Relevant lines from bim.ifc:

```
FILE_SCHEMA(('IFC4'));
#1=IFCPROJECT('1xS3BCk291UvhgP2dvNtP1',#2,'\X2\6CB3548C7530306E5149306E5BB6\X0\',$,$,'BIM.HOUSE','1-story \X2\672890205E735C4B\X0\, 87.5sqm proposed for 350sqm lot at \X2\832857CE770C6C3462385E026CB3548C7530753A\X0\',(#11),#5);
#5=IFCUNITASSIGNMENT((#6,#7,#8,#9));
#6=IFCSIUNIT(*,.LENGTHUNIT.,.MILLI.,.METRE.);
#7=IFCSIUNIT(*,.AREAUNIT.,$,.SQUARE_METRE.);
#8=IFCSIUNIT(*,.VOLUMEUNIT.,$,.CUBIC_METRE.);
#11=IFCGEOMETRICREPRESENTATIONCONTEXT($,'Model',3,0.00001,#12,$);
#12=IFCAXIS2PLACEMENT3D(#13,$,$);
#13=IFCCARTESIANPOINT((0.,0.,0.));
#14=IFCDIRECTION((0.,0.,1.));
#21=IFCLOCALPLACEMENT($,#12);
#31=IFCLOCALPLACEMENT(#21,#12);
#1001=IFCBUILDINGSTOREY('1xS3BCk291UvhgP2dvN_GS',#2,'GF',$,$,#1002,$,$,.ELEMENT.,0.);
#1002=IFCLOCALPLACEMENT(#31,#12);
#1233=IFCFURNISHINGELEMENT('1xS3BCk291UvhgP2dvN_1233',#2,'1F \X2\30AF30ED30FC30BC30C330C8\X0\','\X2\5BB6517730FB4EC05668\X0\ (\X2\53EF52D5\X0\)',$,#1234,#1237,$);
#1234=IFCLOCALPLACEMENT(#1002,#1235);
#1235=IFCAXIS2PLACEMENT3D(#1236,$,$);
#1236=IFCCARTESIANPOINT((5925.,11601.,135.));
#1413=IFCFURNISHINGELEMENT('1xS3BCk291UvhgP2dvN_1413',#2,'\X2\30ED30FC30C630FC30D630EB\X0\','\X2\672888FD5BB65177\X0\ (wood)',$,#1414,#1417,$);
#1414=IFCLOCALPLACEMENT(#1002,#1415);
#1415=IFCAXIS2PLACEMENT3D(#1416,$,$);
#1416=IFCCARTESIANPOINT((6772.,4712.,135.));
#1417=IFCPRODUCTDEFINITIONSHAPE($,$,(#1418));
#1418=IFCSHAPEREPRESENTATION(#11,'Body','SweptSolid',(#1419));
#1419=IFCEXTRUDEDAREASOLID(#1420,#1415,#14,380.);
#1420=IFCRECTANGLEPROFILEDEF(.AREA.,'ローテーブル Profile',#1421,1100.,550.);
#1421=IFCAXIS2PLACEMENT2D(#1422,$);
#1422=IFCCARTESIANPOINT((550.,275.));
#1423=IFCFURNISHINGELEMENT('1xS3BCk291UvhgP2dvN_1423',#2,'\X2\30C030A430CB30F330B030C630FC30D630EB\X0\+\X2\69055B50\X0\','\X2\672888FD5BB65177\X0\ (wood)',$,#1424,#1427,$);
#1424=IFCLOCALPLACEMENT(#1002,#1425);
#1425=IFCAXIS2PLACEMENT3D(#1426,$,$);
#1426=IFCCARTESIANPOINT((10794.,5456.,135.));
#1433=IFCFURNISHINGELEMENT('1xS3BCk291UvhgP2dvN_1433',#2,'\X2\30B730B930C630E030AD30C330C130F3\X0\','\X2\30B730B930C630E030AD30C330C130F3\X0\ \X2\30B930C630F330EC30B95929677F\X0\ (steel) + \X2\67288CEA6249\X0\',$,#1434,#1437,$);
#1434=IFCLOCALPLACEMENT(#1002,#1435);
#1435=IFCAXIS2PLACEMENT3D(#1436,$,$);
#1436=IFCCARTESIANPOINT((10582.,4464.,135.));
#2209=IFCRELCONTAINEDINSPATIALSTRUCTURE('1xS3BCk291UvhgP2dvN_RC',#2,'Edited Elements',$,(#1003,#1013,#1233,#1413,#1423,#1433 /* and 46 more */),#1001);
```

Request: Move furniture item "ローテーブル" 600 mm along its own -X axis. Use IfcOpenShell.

```python
import ifcopenshell
import ifcopenshell.api.geometry
import ifcopenshell.util.placement
import ifcopenshell.util.unit

model = ifcopenshell.open("bim.ifc")
unit_scale = ifcopenshell.util.unit.calculate_unit_scale(model)

item = model.by_id(1413)
matrix = ifcopenshell.util.placement.get_local_placement(item.ObjectPlacement)
matrix[:3, 3] -= matrix[:3, 0] * 0.6 / unit_scale
ifcopenshell.api.geometry.edit_object_placement(model, product=item, matrix=matrix, is_si=False)

print(ifcopenshell.util.placement.get_local_placement(item.ObjectPlacement).round(3) + 0.0)

model.write("bim_updated.ifc")
```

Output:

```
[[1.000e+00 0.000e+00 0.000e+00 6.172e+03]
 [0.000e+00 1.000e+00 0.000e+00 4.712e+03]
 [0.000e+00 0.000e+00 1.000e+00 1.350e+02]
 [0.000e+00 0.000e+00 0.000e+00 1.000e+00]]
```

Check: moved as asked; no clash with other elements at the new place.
